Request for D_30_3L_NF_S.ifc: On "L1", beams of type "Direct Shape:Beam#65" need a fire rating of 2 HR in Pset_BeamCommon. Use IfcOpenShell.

First a look at what the model holds.

```python
import ifcopenshell
import ifcopenshell.util.element

model = ifcopenshell.open("D_30_3L_NF_S.ifc")
print(model.schema)
storey = next(s for s in model.by_type("IfcBuildingStorey") if s.Name == "L1")
beams = [e for e in ifcopenshell.util.element.get_decomposition(storey) if e.is_a("IfcBeam")]
seen = {}
for e in beams:
    element_type = ifcopenshell.util.element.get_type(e)
    key = (element_type.Name if element_type != e and element_type else None, ifcopenshell.util.element.get_pset(e, "Pset_BeamCommon", "FireRating"))
    seen[key] = seen.get(key, 0) + 1
for (name, value), count in sorted(seen.items(), key=str):
    print(count, "x", name, "|", value)
```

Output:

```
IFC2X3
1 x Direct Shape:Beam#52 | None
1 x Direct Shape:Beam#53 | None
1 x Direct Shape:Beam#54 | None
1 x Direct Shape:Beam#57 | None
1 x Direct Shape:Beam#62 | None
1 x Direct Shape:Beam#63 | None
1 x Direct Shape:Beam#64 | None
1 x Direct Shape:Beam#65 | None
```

```python
import ifcopenshell
import ifcopenshell.api.pset
import ifcopenshell.util.element

model = ifcopenshell.open("D_30_3L_NF_S.ifc")

storey = next(s for s in model.by_type("IfcBuildingStorey") if s.Name == "L1")
beams = [e for e in ifcopenshell.util.element.get_decomposition(storey) if e.is_a("IfcBeam")]

count = 0
for e in beams:
    element_type = ifcopenshell.util.element.get_type(e)
    if element_type in (None, e) or element_type.Name != "Direct Shape:Beam#65":
        continue
    # add_pset returns the element's existing set when there is one.
    pset = ifcopenshell.api.pset.add_pset(model, product=e, name="Pset_BeamCommon")
    ifcopenshell.api.pset.edit_pset(model, pset=pset, properties={"FireRating": "2 HR"})
    count += 1

print(count, "beams updated")

model.write("D_30_3L_NF_S-out.ifc")
```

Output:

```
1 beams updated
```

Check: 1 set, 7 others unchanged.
